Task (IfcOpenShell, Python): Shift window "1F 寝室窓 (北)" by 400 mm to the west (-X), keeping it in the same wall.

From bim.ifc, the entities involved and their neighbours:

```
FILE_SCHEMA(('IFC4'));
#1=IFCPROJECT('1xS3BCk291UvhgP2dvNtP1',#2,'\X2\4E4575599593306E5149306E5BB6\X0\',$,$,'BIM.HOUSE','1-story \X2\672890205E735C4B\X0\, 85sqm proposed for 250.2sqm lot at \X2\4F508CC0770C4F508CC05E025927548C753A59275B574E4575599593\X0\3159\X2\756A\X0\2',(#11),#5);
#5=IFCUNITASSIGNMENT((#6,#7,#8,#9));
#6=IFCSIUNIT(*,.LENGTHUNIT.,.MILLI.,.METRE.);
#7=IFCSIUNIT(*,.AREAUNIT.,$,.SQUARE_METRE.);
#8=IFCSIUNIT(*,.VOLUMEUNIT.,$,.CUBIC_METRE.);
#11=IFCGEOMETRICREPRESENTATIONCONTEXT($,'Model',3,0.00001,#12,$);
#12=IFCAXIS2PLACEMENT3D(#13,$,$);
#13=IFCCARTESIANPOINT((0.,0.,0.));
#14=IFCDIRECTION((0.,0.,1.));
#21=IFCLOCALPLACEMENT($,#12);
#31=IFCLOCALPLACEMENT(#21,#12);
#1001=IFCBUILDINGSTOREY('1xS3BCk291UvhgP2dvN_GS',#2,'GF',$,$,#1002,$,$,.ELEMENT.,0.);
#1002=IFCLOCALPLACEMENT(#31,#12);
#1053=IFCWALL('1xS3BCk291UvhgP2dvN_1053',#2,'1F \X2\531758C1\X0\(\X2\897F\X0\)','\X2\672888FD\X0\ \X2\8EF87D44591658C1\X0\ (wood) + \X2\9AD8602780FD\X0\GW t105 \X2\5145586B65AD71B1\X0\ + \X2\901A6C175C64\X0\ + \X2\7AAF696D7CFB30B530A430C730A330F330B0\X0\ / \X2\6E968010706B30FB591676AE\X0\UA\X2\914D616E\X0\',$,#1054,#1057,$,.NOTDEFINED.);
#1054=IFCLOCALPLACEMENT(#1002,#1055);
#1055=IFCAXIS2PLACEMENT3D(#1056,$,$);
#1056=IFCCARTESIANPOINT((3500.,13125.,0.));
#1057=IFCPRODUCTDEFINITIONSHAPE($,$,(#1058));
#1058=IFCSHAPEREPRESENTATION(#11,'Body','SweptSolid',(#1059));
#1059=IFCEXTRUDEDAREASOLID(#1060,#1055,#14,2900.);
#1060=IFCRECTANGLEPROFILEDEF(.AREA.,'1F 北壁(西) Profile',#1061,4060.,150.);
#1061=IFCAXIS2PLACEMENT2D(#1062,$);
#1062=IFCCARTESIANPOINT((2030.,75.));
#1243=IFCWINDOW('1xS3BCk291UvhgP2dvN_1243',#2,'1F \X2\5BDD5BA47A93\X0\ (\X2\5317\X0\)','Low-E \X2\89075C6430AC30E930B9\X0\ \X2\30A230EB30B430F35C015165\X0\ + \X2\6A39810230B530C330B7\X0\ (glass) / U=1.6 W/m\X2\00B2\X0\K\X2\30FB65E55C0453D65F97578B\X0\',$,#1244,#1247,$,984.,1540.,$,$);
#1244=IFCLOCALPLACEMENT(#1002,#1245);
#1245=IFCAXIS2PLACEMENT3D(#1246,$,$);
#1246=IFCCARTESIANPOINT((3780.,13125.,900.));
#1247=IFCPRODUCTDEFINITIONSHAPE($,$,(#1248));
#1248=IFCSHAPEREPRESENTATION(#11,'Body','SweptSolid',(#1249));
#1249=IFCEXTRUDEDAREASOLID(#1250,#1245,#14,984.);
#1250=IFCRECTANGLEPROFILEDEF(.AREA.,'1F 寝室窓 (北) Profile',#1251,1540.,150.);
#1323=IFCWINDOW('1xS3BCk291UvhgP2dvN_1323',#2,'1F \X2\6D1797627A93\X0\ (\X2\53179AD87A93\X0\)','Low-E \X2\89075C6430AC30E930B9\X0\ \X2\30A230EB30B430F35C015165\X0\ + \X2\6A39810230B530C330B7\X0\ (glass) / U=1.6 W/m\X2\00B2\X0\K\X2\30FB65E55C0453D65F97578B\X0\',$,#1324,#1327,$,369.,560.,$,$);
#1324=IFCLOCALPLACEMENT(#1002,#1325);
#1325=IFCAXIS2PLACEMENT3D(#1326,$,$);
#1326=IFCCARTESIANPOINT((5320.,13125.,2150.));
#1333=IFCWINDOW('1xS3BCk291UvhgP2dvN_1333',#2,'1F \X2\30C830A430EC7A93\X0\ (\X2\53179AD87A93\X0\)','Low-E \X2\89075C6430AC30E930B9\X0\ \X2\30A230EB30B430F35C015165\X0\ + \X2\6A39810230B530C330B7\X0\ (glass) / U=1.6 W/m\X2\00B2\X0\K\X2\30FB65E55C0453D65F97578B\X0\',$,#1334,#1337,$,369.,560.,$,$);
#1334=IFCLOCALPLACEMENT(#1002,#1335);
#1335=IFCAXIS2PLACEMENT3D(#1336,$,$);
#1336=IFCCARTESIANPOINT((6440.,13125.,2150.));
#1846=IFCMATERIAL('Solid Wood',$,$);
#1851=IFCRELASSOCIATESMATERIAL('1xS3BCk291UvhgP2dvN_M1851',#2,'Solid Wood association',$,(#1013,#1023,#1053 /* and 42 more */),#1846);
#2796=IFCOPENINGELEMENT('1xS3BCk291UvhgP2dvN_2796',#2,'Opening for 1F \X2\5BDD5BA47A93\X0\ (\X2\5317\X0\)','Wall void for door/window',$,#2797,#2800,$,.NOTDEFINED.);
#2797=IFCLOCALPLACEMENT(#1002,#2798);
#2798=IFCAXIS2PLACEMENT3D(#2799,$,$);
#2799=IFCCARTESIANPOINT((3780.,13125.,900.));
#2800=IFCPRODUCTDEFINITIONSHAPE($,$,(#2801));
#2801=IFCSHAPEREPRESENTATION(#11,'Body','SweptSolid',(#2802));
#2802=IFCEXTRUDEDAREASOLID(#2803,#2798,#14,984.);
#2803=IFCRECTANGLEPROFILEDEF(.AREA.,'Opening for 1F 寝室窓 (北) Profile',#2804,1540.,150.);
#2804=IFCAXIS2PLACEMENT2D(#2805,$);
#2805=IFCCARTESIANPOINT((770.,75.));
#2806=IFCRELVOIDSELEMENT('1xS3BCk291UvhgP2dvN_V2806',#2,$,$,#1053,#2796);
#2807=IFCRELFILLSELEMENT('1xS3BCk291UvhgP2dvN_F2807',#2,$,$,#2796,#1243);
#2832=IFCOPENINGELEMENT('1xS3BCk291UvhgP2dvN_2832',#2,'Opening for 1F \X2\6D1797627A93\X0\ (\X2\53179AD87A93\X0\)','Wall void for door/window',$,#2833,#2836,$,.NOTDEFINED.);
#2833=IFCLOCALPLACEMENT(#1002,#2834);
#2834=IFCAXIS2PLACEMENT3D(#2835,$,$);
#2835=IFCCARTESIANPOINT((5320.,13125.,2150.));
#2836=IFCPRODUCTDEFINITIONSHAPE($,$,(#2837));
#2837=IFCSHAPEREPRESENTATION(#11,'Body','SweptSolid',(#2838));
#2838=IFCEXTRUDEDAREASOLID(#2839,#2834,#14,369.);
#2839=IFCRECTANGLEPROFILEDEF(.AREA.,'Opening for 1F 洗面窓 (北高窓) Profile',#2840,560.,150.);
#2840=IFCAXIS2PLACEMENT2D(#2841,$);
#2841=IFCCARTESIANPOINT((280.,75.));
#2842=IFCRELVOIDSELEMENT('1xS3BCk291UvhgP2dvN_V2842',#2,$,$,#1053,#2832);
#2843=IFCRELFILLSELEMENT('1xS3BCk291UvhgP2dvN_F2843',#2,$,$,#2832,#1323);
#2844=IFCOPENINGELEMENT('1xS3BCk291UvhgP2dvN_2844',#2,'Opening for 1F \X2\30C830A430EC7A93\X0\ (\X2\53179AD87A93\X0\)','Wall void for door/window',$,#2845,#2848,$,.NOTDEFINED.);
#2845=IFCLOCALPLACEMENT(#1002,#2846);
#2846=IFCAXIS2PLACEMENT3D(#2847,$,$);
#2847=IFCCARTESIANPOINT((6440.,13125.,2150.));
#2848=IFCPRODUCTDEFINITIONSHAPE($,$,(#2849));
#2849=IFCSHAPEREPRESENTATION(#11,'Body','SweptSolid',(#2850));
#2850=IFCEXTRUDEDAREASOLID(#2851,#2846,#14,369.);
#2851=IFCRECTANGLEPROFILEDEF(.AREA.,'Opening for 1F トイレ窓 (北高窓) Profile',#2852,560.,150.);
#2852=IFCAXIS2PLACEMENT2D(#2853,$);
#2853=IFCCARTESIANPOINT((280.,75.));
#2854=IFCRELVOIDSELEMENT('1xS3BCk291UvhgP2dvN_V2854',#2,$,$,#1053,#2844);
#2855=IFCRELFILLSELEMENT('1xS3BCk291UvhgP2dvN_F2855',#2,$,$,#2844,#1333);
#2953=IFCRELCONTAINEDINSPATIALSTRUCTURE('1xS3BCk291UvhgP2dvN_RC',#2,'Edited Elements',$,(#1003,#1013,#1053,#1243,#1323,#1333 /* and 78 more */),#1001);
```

```python
import ifcopenshell
import ifcopenshell.api.geometry
import ifcopenshell.util.placement

model = ifcopenshell.open("bim.ifc")

window = model.by_guid("1xS3BCk291UvhgP2dvN_1243")
opening = window.FillsVoids[0].RelatingOpeningElement
wall = opening.VoidsElements[0].RelatingBuildingElement

wall_matrix = ifcopenshell.util.placement.get_local_placement(wall.ObjectPlacement)
shift = wall_matrix[:3, 0] * -400.0
before = ifcopenshell.util.placement.get_local_placement(window.ObjectPlacement)[:3, 3].copy()

# The window is not placed relative to its opening, so move both.
for product in (opening, window):
    matrix = ifcopenshell.util.placement.get_local_placement(product.ObjectPlacement)
    matrix[:3, 3] += shift
    ifcopenshell.api.geometry.edit_object_placement(model, product=product, matrix=matrix, is_si=False)

after = ifcopenshell.util.placement.get_local_placement(window.ObjectPlacement)[:3, 3]
print("window moved by", (after - before).round(3) + 0.0)

model.write("bim_updated.ifc")
```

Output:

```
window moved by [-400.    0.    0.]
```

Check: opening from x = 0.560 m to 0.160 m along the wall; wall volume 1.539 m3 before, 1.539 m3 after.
